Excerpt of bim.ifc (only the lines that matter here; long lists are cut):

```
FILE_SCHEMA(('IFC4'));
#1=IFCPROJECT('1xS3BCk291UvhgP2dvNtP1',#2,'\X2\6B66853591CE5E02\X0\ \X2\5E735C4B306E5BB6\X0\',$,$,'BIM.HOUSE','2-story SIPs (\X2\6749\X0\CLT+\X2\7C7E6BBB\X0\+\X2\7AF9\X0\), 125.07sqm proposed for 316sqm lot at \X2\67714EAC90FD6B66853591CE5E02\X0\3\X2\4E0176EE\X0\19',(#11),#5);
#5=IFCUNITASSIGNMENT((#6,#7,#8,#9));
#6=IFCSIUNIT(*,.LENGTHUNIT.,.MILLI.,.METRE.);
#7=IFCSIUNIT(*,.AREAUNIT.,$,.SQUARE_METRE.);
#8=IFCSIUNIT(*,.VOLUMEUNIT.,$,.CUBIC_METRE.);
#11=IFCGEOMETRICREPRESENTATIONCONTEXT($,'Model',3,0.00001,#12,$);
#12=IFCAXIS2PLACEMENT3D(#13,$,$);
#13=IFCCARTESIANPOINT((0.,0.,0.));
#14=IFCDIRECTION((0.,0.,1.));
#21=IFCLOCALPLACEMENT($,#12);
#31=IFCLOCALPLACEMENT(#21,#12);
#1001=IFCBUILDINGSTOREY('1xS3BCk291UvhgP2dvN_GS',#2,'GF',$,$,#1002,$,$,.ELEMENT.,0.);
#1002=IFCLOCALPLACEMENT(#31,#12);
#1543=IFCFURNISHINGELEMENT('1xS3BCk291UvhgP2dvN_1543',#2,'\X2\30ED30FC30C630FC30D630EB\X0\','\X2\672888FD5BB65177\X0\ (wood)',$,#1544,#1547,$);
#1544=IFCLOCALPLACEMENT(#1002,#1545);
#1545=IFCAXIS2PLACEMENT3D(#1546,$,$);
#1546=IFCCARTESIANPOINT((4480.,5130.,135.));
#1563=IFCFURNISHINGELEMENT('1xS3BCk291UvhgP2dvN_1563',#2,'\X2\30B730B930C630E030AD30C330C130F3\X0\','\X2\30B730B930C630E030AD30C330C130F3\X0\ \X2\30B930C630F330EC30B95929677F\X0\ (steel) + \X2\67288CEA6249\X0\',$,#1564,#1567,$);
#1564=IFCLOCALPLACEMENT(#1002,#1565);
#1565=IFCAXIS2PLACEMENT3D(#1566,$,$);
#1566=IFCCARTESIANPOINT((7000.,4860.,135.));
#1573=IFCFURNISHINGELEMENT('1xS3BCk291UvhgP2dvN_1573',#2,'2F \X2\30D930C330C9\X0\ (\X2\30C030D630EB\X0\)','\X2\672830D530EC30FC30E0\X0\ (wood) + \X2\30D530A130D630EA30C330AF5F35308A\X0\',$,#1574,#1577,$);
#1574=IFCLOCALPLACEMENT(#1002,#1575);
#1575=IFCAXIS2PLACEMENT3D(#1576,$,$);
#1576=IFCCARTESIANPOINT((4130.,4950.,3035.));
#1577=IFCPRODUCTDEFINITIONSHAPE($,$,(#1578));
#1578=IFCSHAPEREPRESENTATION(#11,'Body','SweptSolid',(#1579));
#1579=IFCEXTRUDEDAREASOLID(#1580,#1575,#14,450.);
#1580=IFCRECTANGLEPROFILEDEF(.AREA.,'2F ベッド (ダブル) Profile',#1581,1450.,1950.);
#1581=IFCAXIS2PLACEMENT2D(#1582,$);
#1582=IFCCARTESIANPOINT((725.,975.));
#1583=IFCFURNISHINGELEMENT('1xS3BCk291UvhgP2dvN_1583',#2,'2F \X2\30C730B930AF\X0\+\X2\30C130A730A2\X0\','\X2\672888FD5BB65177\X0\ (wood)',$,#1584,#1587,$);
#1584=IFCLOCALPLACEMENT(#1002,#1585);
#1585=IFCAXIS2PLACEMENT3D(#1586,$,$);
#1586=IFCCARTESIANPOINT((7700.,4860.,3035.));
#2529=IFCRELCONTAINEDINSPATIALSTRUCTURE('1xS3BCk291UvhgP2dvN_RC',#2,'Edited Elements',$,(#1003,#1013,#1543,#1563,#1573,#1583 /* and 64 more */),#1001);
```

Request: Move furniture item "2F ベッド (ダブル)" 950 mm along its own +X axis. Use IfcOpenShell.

```python
import ifcopenshell
import ifcopenshell.api.geometry
import ifcopenshell.util.placement
import ifcopenshell.util.unit

model = ifcopenshell.open("bim.ifc")
unit_scale = ifcopenshell.util.unit.calculate_unit_scale(model)

item = model.by_guid("1xS3BCk291UvhgP2dvN_1573")
matrix = ifcopenshell.util.placement.get_local_placement(item.ObjectPlacement)
matrix[:3, 3] += matrix[:3, 0] * 0.95 / unit_scale
ifcopenshell.api.geometry.edit_object_placement(model, product=item, matrix=matrix, is_si=False)

print(ifcopenshell.util.placement.get_local_placement(item.ObjectPlacement).round(3) + 0.0)

model.write("bim_updated.ifc")
```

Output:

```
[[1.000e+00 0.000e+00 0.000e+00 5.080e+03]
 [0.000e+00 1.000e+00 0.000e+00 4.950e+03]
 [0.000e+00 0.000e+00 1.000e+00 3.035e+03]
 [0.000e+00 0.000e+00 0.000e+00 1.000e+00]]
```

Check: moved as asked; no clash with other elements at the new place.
